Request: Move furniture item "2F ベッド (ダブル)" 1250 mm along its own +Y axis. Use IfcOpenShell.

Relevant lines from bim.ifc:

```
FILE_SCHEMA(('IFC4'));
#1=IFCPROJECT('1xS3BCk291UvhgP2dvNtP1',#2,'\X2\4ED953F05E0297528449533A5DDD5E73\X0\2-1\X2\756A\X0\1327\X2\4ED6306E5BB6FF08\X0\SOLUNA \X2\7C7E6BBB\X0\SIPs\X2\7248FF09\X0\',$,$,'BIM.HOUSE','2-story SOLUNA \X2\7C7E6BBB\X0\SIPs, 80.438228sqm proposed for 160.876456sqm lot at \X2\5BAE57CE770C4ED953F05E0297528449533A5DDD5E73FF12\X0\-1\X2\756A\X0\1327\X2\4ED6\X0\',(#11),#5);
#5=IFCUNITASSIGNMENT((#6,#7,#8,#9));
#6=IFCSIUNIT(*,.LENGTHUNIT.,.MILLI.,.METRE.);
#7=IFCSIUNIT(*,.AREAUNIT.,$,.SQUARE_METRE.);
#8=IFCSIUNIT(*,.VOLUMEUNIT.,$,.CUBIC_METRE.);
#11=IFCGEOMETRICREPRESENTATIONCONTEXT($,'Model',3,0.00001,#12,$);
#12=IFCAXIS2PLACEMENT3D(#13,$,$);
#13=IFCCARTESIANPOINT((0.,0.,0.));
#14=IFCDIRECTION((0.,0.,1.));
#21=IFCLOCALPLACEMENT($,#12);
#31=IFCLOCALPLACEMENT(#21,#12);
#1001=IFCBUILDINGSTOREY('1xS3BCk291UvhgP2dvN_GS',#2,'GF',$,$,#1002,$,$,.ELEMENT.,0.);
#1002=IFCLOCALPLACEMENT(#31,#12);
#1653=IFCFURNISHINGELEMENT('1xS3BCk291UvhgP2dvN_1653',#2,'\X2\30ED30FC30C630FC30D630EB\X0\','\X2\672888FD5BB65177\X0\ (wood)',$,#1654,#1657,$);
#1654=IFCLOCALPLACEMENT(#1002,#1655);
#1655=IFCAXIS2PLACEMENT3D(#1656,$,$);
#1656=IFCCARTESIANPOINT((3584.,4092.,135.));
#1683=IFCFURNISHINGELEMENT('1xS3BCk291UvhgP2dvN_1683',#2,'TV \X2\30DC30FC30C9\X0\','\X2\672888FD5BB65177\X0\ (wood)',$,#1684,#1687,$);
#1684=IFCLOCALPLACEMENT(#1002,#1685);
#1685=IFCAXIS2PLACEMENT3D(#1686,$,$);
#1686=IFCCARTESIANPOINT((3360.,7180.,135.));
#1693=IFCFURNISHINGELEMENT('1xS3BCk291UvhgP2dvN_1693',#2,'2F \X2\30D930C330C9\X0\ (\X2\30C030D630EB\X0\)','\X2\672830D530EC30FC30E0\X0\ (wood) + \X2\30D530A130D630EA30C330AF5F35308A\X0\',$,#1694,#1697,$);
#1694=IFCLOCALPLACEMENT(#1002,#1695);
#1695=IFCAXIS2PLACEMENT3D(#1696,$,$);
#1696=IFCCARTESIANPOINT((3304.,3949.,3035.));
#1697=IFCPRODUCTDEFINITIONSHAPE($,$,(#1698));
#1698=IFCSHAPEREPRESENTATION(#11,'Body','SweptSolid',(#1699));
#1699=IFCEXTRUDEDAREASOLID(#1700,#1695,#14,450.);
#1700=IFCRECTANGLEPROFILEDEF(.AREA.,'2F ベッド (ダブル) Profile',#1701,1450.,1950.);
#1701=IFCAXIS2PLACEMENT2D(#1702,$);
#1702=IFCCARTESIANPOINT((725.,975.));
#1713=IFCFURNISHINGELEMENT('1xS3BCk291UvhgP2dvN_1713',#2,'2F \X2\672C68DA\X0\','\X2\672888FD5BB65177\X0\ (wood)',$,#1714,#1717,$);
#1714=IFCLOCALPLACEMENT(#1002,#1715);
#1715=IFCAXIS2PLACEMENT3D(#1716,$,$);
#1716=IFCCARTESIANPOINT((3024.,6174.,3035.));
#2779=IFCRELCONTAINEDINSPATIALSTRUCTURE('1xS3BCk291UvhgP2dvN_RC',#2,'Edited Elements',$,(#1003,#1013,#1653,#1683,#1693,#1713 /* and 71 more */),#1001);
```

```python
import ifcopenshell
import ifcopenshell.api.geometry
import ifcopenshell.util.placement

model = ifcopenshell.open("bim.ifc")

item = model.by_guid("1xS3BCk291UvhgP2dvN_1693")
matrix = ifcopenshell.util.placement.get_local_placement(item.ObjectPlacement)
matrix[:3, 3] += matrix[:3, 1] * 1250.0
ifcopenshell.api.geometry.edit_object_placement(model, product=item, matrix=matrix, is_si=False)

print(ifcopenshell.util.placement.get_local_placement(item.ObjectPlacement).round(3) + 0.0)

model.write("bim_updated.ifc")
```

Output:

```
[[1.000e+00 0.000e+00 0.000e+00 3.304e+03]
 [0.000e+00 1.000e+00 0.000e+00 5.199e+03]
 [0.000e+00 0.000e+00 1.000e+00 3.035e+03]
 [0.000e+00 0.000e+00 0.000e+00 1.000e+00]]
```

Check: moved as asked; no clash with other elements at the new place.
